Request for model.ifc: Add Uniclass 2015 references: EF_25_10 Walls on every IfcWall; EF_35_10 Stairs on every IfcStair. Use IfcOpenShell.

First a look at what the model holds.

```python
import ifcopenshell

model = ifcopenshell.open("model.ifc")
print(model.schema)
print("classifications:", [c.Name for c in model.by_type("IfcClassification")])
for ifc_class in ("IfcDoor", "IfcRoof", "IfcStair", "IfcWall", "IfcWindow"):
    print(ifc_class, len(model.by_type(ifc_class)))
```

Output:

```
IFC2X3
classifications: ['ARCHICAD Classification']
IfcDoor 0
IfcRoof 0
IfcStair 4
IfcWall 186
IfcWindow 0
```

```python
import ifcopenshell
import ifcopenshell.api.classification

model = ifcopenshell.open("model.ifc")

# IFC2X3 requires Source and Edition and has no link from the project to the system.
system = model.create_entity("IfcClassification", Source="NBS", Edition="2015", Name="Uniclass 2015")

codes = {
    "IfcWall": ("EF_25_10", "Walls"),
    "IfcStair": ("EF_35_10", "Stairs"),
}
for ifc_class, (code, name) in codes.items():
    products = model.by_type(ifc_class)
    ifcopenshell.api.classification.add_reference(
        model, products=products, classification=system, identification=code, name=name
    )
    print(code, len(products))

model.write("model_v2.ifc")
```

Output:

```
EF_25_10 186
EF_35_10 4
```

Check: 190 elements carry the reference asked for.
